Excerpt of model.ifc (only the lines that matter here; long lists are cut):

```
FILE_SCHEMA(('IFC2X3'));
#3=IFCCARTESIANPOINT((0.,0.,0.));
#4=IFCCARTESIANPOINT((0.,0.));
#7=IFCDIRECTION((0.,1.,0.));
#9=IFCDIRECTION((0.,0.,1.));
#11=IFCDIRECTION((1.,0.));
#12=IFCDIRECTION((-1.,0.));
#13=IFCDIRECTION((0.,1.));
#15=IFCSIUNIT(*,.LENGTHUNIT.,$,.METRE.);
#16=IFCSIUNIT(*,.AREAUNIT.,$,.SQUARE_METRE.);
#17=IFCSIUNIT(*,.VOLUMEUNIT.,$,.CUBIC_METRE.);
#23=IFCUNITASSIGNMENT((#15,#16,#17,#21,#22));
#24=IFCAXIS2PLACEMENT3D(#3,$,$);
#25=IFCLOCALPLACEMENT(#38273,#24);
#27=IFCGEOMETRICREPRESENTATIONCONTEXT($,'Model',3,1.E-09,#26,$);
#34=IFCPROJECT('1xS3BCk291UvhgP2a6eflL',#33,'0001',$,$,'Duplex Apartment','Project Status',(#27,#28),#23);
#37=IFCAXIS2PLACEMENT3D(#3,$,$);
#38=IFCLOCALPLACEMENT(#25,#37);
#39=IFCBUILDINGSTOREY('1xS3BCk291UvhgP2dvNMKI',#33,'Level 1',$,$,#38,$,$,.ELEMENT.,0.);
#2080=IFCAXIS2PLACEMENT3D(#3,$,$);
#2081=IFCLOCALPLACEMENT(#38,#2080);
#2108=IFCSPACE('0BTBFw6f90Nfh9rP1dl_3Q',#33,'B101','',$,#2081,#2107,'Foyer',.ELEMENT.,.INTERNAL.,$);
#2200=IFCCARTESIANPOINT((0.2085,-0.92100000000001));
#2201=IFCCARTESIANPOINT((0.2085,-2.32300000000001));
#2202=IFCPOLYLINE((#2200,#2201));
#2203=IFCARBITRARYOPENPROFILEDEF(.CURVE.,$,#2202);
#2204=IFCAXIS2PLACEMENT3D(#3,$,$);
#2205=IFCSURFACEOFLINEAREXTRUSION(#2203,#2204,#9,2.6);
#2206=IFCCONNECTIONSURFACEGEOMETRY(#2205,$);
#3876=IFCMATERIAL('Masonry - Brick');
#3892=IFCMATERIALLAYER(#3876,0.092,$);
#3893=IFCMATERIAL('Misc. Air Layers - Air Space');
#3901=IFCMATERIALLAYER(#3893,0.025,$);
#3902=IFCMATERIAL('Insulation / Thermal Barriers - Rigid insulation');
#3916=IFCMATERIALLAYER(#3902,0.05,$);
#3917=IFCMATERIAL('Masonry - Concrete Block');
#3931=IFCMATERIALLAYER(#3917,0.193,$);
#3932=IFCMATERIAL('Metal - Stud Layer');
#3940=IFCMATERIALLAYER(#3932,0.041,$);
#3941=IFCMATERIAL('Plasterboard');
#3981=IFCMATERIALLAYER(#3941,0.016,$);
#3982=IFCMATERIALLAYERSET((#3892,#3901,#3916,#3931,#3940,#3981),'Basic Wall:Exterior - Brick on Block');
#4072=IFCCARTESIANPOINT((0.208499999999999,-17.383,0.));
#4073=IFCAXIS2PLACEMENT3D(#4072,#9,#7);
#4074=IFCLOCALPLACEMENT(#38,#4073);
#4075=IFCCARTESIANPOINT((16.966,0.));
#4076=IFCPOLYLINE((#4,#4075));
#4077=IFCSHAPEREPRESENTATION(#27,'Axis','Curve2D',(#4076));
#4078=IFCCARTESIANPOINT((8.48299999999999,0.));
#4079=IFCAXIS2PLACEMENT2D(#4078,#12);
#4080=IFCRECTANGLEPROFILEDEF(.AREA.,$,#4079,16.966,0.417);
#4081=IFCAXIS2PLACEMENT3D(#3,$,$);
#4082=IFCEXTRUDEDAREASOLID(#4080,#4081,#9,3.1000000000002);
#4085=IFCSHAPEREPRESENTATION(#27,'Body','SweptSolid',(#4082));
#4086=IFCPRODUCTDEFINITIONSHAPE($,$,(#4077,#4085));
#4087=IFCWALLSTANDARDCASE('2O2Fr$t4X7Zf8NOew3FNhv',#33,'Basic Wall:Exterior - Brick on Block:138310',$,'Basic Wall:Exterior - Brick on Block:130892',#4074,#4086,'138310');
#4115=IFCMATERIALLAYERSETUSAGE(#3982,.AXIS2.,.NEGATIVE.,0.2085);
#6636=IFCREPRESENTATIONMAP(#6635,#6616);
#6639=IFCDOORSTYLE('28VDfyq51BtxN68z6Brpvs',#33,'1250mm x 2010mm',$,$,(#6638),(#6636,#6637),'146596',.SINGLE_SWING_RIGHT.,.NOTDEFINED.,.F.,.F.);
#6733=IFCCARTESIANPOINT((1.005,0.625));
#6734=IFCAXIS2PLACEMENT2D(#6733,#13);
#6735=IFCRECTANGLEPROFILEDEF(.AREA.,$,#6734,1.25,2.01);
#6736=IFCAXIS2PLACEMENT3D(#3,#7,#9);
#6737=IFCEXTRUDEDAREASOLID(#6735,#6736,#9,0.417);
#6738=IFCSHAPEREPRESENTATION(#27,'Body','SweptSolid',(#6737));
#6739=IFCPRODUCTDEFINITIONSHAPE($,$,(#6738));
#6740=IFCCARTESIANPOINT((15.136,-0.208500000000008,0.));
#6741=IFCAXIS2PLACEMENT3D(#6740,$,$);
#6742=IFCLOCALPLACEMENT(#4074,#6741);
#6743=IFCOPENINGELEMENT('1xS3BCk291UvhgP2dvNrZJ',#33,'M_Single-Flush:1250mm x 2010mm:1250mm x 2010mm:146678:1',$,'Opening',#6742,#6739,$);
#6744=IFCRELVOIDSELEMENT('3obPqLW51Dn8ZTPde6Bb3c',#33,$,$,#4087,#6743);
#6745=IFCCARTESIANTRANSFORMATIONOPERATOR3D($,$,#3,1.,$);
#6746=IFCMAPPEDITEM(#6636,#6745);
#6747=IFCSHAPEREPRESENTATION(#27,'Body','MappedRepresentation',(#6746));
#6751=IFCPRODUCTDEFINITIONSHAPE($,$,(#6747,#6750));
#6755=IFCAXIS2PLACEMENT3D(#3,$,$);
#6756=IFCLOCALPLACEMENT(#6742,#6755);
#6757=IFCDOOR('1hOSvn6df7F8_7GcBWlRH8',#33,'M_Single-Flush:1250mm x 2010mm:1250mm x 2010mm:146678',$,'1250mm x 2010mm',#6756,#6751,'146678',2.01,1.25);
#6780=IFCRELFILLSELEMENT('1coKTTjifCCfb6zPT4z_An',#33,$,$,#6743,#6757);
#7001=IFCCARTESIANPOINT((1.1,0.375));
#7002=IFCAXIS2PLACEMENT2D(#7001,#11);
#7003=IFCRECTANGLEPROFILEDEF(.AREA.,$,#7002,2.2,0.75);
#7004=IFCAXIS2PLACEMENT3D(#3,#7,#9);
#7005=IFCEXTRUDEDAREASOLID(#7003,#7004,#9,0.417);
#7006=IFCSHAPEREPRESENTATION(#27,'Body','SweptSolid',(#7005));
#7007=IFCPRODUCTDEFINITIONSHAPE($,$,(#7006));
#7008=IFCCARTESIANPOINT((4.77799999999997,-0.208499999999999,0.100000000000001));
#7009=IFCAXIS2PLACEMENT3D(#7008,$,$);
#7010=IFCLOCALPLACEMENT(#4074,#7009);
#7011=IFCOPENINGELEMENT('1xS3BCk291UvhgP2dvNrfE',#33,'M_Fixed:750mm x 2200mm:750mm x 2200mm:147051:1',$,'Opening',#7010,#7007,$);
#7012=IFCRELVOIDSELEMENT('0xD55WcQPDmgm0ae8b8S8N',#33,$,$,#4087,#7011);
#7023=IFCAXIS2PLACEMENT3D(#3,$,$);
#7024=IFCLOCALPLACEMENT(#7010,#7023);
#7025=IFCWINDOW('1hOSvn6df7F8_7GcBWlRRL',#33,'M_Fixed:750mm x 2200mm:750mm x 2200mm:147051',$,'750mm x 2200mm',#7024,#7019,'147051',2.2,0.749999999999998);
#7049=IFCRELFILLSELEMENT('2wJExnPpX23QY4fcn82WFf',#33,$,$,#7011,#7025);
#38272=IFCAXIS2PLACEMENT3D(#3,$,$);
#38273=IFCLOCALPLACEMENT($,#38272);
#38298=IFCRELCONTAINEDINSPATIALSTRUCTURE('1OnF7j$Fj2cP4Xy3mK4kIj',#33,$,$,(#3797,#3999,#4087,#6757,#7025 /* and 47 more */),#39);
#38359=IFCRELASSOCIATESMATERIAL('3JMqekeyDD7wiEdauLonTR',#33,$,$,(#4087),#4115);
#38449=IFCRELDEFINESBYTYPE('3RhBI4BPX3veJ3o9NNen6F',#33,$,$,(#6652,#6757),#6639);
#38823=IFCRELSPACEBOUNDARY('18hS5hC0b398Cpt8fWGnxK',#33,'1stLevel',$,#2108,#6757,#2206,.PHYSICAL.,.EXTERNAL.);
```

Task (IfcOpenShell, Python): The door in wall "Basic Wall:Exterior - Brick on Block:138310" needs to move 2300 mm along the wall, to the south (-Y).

```python
import numpy as np
import ifcopenshell
import ifcopenshell.api.geometry
import ifcopenshell.util.placement
import ifcopenshell.util.unit

model = ifcopenshell.open("model.ifc")
unit_scale = ifcopenshell.util.unit.calculate_unit_scale(model)

door = model.by_guid("1hOSvn6df7F8_7GcBWlRH8")
opening = door.FillsVoids[0].RelatingOpeningElement
wall = opening.VoidsElements[0].RelatingBuildingElement

wall_matrix = ifcopenshell.util.placement.get_local_placement(wall.ObjectPlacement)
shift = wall_matrix[:3, 0] * -2.3 / unit_scale
before = ifcopenshell.util.placement.get_local_placement(door.ObjectPlacement)[:3, 3].copy()

# The door is placed relative to its opening, so it follows when the opening moves.
matrix = ifcopenshell.util.placement.get_local_placement(opening.ObjectPlacement)
matrix[:3, 3] += shift
ifcopenshell.api.geometry.edit_object_placement(
    model, product=opening, matrix=matrix, is_si=False, should_transform_children=True
)

# Space boundary surfaces are stored in each space's coordinates; move them too.
for rel in door.ProvidesBoundaries:
    if not rel.ConnectionGeometry:
        continue
    surface = rel.ConnectionGeometry.SurfaceOnRelatingElement
    space_matrix = ifcopenshell.util.placement.get_local_placement(rel.RelatingSpace.ObjectPlacement)
    point = np.array(surface.Position.Location.Coordinates) + space_matrix[:3, :3].T @ shift
    surface.Position = model.createIfcAxis2Placement3D(
        model.createIfcCartesianPoint(point.tolist()), surface.Position.Axis, surface.Position.RefDirection
    )

after = ifcopenshell.util.placement.get_local_placement(door.ObjectPlacement)[:3, 3]
print("door moved by", (after - before).round(3) + 0.0)

model.write("model-out.ifc")
```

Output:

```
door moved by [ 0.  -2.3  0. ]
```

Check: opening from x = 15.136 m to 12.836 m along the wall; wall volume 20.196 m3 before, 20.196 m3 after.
